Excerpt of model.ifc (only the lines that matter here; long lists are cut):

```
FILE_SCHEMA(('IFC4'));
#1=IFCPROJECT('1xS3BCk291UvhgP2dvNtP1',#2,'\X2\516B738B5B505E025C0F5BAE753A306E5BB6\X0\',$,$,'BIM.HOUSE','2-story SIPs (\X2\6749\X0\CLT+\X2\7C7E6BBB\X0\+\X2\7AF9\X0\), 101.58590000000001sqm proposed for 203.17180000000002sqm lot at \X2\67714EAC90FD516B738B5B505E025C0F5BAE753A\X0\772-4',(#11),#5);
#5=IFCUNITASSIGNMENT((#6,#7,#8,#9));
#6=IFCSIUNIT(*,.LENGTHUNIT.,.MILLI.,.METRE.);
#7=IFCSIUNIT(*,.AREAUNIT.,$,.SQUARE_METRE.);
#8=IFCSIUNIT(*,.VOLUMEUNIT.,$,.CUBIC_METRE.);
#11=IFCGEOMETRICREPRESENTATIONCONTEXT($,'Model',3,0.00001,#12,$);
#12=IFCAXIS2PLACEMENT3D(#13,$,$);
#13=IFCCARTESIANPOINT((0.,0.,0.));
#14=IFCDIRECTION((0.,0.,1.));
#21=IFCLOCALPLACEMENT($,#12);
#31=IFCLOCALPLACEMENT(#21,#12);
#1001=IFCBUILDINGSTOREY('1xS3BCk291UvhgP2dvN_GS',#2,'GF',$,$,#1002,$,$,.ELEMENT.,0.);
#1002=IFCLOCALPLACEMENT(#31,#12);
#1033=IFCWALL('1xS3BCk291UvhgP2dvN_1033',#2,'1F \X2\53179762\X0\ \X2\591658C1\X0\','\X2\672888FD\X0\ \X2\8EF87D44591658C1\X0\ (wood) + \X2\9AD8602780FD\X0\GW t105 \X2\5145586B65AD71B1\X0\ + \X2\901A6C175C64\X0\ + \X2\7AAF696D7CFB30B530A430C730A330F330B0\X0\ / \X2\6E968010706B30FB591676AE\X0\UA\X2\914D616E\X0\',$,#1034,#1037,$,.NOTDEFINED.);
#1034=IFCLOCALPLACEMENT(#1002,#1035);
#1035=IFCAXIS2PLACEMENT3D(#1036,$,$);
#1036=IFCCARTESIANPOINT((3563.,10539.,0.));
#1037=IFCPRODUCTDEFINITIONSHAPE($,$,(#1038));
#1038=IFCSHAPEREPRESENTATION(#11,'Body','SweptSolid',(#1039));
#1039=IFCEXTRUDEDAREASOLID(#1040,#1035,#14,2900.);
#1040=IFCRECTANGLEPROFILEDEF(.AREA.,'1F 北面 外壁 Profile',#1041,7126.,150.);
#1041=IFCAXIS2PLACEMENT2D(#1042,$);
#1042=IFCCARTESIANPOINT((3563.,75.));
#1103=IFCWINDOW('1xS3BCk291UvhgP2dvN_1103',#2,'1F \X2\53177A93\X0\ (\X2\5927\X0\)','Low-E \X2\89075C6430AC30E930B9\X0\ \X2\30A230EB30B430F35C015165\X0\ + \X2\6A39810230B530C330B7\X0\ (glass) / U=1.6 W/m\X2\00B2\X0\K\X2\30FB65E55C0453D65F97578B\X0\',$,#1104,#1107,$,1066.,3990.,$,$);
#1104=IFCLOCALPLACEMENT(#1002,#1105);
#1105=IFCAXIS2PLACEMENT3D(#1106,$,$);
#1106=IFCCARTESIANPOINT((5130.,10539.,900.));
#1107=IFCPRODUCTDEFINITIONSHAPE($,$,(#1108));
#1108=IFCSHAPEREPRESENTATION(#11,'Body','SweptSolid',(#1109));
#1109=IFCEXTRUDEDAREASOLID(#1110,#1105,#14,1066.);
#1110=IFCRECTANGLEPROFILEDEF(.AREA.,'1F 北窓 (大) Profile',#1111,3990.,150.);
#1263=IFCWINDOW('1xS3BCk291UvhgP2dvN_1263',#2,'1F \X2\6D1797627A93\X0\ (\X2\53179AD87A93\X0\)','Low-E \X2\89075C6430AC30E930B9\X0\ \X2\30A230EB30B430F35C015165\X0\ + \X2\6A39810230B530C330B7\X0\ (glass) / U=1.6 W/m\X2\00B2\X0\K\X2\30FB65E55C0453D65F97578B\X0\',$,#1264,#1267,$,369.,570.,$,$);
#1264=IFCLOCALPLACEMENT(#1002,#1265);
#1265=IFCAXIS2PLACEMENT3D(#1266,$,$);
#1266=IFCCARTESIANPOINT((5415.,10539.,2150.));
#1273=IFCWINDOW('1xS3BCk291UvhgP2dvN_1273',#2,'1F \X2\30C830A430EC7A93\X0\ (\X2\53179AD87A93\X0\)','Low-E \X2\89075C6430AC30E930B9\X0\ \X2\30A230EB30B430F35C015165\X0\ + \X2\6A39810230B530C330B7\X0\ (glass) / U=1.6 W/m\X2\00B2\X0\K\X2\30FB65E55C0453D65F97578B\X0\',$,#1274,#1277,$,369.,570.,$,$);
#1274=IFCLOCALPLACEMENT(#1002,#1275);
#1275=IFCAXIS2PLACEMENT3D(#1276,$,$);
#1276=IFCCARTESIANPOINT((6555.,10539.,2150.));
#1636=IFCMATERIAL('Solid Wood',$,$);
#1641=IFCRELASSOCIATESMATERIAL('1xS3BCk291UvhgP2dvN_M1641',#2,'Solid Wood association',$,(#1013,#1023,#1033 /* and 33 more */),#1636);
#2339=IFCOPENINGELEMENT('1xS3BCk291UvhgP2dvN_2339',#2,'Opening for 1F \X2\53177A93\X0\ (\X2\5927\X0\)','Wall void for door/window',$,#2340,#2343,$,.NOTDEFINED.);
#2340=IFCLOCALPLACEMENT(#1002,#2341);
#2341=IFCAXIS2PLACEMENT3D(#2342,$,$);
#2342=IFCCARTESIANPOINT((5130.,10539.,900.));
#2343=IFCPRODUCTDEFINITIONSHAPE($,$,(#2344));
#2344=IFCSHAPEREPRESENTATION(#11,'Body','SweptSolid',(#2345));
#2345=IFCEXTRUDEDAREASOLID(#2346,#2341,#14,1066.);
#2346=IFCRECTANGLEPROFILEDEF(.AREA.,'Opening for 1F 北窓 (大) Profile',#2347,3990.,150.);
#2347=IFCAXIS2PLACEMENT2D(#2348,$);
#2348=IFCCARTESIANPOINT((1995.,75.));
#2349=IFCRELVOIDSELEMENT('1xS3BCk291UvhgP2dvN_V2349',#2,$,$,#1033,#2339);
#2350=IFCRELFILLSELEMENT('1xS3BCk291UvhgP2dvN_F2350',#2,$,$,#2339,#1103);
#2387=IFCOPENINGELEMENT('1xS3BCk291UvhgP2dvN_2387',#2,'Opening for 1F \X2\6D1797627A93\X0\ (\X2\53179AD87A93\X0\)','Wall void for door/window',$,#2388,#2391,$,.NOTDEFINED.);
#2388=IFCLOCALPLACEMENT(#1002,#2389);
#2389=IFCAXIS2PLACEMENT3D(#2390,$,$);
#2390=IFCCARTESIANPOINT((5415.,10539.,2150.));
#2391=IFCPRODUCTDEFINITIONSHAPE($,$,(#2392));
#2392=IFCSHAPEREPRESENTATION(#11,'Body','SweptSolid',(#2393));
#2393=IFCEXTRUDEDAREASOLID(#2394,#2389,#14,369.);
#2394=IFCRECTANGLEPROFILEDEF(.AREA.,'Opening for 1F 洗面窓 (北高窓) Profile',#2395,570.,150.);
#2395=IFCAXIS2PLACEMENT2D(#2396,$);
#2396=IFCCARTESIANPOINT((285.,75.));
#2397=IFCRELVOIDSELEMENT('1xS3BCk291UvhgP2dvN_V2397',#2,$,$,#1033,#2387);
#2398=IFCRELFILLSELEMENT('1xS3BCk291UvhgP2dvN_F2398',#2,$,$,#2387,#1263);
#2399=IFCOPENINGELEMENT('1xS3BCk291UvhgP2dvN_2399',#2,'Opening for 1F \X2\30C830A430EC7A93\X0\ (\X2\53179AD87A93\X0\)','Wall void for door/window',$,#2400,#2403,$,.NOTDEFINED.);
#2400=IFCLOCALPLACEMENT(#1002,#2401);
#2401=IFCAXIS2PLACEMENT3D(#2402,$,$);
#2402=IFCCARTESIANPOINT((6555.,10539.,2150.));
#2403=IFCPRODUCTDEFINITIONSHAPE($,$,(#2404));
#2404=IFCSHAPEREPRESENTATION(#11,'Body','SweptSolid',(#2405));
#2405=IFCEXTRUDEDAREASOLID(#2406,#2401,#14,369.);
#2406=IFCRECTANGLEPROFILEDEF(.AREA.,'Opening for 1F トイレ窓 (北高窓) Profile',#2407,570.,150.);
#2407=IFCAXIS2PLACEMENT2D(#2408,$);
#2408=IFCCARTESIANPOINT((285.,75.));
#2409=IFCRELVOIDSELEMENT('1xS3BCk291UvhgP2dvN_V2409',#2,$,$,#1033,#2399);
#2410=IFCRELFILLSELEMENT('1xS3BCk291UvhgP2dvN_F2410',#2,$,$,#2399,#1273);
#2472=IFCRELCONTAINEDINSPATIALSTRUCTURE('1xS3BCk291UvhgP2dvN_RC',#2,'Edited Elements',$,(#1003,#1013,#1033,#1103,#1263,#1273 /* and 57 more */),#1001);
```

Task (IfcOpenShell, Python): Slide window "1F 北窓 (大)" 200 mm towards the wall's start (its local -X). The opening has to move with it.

```python
import ifcopenshell
import ifcopenshell.api.geometry
import ifcopenshell.util.placement

model = ifcopenshell.open("model.ifc")

window = model.by_guid("1xS3BCk291UvhgP2dvN_1103")
opening = window.FillsVoids[0].RelatingOpeningElement
wall = opening.VoidsElements[0].RelatingBuildingElement

wall_matrix = ifcopenshell.util.placement.get_local_placement(wall.ObjectPlacement)
shift = wall_matrix[:3, 0] * -200.0
before = ifcopenshell.util.placement.get_local_placement(window.ObjectPlacement)[:3, 3].copy()

# The window is not placed relative to its opening, so move both.
for product in (opening, window):
    matrix = ifcopenshell.util.placement.get_local_placement(product.ObjectPlacement)
    matrix[:3, 3] += shift
    ifcopenshell.api.geometry.edit_object_placement(model, product=product, matrix=matrix, is_si=False)

after = ifcopenshell.util.placement.get_local_placement(window.ObjectPlacement)[:3, 3]
print("window moved by", (after - before).round(3) + 0.0)

model.write("model_rev.ifc")
```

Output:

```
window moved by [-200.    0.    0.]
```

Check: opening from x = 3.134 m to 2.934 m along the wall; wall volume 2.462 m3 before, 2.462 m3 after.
